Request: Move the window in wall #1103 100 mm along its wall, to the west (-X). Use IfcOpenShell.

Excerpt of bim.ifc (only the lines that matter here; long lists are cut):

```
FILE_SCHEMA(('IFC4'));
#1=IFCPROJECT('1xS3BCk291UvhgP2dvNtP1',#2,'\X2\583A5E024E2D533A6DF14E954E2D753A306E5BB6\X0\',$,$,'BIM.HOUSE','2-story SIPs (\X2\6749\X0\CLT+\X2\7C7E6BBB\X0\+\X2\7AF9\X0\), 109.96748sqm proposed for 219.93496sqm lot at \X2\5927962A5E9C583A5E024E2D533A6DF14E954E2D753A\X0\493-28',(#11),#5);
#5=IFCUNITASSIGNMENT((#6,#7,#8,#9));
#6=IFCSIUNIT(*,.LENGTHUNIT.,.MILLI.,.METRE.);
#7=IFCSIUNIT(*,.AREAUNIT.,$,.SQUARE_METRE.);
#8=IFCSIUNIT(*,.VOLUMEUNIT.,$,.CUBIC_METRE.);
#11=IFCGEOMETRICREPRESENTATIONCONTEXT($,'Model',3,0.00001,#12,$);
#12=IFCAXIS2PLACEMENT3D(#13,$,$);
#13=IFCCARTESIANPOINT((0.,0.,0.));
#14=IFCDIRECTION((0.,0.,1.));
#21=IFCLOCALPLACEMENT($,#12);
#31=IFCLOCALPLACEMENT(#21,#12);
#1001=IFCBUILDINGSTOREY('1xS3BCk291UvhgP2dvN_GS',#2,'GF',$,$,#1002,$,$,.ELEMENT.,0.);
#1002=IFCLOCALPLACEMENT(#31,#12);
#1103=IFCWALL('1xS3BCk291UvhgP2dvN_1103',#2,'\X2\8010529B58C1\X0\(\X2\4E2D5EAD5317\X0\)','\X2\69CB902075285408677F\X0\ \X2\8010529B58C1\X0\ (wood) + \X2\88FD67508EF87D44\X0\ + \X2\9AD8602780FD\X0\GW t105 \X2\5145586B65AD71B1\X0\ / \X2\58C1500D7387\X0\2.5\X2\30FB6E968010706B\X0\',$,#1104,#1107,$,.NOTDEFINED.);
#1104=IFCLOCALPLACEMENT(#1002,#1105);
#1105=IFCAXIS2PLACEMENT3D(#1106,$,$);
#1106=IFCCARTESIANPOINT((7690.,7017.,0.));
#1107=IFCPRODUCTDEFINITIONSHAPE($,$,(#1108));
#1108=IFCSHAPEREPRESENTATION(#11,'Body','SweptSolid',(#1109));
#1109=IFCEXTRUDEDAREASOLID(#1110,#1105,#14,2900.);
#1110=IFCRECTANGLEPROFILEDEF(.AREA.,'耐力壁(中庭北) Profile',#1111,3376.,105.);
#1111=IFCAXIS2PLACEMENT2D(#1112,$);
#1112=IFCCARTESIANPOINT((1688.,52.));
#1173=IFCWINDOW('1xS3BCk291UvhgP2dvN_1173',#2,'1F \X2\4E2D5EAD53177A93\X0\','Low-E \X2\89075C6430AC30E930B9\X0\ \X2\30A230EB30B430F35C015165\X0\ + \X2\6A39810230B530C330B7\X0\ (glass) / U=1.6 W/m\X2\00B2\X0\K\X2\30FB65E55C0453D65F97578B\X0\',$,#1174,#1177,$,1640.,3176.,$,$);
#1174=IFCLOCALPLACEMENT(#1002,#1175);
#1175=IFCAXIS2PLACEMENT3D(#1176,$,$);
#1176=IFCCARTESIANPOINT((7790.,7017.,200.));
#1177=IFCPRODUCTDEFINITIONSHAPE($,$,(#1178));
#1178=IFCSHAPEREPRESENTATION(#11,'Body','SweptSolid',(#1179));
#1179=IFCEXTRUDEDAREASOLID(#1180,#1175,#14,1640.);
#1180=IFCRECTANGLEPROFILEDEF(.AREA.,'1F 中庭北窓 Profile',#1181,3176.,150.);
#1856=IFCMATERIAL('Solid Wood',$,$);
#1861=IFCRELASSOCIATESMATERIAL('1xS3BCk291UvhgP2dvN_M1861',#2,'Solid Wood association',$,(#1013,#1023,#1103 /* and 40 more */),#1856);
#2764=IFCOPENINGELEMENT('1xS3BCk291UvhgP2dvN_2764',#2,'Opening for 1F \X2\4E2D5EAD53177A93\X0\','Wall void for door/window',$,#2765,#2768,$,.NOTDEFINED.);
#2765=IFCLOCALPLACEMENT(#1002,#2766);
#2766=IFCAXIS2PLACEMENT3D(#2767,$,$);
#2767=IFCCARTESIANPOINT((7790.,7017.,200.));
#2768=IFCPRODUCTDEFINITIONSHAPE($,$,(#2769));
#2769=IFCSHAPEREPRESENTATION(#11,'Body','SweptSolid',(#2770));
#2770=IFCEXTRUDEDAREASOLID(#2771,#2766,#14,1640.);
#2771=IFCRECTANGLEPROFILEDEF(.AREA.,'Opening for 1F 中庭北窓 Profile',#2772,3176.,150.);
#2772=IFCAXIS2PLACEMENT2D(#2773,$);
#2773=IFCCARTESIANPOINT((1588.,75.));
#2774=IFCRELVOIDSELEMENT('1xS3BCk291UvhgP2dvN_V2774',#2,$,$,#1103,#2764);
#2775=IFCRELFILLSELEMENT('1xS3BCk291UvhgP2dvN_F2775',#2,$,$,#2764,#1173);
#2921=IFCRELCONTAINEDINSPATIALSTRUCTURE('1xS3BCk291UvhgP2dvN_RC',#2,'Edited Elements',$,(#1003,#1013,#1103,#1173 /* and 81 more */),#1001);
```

```python
import ifcopenshell
import ifcopenshell.api.geometry
import ifcopenshell.util.placement
import ifcopenshell.util.unit

model = ifcopenshell.open("bim.ifc")
unit_scale = ifcopenshell.util.unit.calculate_unit_scale(model)

window = model.by_guid("1xS3BCk291UvhgP2dvN_1173")
opening = window.FillsVoids[0].RelatingOpeningElement
wall = opening.VoidsElements[0].RelatingBuildingElement

wall_matrix = ifcopenshell.util.placement.get_local_placement(wall.ObjectPlacement)
shift = wall_matrix[:3, 0] * -0.1 / unit_scale
before = ifcopenshell.util.placement.get_local_placement(window.ObjectPlacement)[:3, 3].copy()

# The window is not placed relative to its opening, so move both.
for product in (opening, window):
    matrix = ifcopenshell.util.placement.get_local_placement(product.ObjectPlacement)
    matrix[:3, 3] += shift
    ifcopenshell.api.geometry.edit_object_placement(model, product=product, matrix=matrix, is_si=False)

after = ifcopenshell.util.placement.get_local_placement(window.ObjectPlacement)[:3, 3]
print("window moved by", (after - before).round(3) + 0.0)

model.write("bim_v2.ifc")
```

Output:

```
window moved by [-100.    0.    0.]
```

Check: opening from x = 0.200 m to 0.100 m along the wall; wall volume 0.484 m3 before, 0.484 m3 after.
